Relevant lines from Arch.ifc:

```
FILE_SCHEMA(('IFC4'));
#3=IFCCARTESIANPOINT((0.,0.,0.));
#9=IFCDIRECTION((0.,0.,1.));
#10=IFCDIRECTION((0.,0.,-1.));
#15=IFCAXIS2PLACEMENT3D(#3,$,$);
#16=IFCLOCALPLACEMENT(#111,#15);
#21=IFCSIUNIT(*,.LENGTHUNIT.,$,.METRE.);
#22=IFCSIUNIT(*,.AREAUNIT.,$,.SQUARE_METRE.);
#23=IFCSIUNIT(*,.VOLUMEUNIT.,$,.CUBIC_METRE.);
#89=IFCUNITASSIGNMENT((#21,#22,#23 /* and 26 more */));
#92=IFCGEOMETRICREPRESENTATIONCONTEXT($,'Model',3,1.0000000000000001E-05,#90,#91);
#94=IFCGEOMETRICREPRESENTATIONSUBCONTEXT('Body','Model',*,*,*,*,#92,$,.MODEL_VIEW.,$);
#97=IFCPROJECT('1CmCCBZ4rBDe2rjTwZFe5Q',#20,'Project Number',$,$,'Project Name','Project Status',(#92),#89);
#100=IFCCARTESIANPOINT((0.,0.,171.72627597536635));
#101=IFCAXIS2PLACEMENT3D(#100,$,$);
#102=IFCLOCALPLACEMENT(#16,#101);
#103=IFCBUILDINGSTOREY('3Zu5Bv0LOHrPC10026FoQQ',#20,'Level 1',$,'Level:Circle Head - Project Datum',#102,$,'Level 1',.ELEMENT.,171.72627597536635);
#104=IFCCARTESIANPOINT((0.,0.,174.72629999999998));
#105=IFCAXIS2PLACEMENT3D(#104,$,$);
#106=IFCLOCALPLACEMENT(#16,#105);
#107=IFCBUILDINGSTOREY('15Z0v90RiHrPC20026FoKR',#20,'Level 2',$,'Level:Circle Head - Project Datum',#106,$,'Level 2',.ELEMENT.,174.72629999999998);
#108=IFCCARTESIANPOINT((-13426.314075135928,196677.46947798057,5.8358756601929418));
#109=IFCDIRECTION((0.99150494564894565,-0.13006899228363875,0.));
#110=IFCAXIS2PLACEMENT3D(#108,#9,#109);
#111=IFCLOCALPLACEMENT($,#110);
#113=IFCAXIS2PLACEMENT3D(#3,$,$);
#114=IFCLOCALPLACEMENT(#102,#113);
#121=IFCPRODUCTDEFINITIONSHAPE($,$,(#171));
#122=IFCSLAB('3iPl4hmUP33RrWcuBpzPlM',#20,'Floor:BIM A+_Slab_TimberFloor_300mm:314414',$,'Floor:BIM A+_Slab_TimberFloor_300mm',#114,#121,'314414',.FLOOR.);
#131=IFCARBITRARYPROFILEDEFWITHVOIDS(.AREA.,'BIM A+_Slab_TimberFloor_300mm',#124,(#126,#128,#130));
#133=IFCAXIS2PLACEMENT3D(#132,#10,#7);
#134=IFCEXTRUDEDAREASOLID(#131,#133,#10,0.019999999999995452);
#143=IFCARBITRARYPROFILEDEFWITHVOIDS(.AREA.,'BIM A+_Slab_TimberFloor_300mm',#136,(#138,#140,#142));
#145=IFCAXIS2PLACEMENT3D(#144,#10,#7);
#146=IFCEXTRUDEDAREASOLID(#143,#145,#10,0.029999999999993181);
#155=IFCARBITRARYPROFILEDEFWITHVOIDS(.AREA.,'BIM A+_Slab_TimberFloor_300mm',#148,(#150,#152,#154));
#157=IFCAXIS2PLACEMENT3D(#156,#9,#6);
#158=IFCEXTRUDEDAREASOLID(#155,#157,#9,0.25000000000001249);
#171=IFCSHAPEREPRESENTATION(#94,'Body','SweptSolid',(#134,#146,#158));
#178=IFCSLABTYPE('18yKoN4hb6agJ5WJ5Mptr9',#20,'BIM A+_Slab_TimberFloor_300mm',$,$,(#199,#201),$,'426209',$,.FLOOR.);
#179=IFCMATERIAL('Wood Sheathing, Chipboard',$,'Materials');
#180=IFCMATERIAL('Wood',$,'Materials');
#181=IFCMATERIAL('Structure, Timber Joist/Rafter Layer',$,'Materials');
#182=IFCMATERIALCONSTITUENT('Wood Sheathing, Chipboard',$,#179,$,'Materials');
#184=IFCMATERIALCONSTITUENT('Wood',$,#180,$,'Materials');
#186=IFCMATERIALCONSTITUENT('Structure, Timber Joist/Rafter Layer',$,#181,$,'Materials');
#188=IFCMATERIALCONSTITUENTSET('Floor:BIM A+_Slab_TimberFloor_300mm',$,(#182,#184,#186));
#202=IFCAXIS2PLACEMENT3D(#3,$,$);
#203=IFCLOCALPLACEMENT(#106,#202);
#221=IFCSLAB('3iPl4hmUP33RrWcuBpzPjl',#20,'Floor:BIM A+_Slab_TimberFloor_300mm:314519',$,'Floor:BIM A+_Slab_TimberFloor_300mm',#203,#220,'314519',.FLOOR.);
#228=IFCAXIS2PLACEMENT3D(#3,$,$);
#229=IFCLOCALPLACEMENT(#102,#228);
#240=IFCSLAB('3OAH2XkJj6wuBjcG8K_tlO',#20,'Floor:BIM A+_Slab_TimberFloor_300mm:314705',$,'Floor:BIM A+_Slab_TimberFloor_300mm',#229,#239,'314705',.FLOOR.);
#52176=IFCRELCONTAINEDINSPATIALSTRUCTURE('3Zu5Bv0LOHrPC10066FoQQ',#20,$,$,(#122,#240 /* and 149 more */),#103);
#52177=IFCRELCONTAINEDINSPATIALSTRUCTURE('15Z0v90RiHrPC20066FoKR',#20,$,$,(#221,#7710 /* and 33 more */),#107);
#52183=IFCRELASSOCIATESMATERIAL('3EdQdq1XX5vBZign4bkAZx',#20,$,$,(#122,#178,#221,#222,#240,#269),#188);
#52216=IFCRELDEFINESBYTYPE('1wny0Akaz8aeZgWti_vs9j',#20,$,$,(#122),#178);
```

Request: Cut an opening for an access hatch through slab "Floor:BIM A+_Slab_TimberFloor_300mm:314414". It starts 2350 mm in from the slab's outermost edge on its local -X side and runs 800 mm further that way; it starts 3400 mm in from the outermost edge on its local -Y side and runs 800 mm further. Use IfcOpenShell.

```python
import numpy as np
import ifcopenshell
import ifcopenshell.api.feature
import ifcopenshell.api.geometry
import ifcopenshell.api.root
import ifcopenshell.geom
import ifcopenshell.util.placement
import ifcopenshell.util.representation
import ifcopenshell.util.shape
import ifcopenshell.util.unit

model = ifcopenshell.open("Arch.ifc")
unit_scale = ifcopenshell.util.unit.calculate_unit_scale(model)
settings = ifcopenshell.geom.settings()


def volume(element):
    """Net volume in cubic metres, openings subtracted."""
    shape = ifcopenshell.geom.create_shape(settings, element)
    return ifcopenshell.util.shape.get_volume(shape.geometry)


slab = model.by_guid("3iPl4hmUP33RrWcuBpzPlM")
before = volume(slab)

# Extent in the slab's own axes, in metres. The edges named are its -X and -Y sides.
slab_shape = ifcopenshell.geom.create_shape(settings, slab)
vertices = ifcopenshell.util.shape.get_vertices(slab_shape.geometry)
x_min, y_min, bottom = vertices.min(axis=0)
top = vertices[:, 2].max()

opening = ifcopenshell.api.root.create_entity(model, ifc_class="IfcOpeningElement", name="Access hatch opening", predefined_type="OPENING")
context = ifcopenshell.util.representation.get_context(model, "Model", "Body", "MODEL_VIEW")
width, depth = 0.8, 0.8
outline = [(0.0, 0.0), (width, 0.0), (width, depth), (0.0, depth), (0.0, 0.0)]
# Overshoot both faces by 50 mm so the cut is clean.
shape = ifcopenshell.api.geometry.add_slab_representation(
    model, context=context, depth=top - bottom + 0.1, polyline=outline
)
ifcopenshell.api.geometry.assign_representation(model, product=opening, representation=shape)

matrix = ifcopenshell.util.placement.get_local_placement(slab.ObjectPlacement)
matrix[:, 3] = matrix @ np.append(np.array([x_min + 2.35, y_min + 3.4, bottom - 0.05]) / unit_scale, 1.0)
ifcopenshell.api.geometry.edit_object_placement(model, product=opening, matrix=matrix, is_si=False)
ifcopenshell.api.feature.add_feature(model, feature=opening, element=slab)

after = volume(slab)

print(f"slab volume {before:.3f} -> {after:.3f} m3")

model.write("Arch_edited.ifc")
```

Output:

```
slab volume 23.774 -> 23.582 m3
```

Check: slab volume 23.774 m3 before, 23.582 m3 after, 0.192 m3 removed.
